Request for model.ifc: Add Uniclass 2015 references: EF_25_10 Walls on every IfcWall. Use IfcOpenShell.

First a look at what the model holds.

```python
import ifcopenshell

model = ifcopenshell.open("model.ifc")
print(model.schema)
print("classifications:", [c.Name for c in model.by_type("IfcClassification")])
for ifc_class in ("IfcDoor", "IfcRoof", "IfcStair", "IfcWall", "IfcWindow"):
    print(ifc_class, len(model.by_type(ifc_class)))
```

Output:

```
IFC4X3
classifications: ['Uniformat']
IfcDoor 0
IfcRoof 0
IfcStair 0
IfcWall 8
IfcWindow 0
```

```python
import ifcopenshell
import ifcopenshell.api.classification

model = ifcopenshell.open("model.ifc")

system = ifcopenshell.api.classification.add_classification(model, classification="Uniclass 2015")

codes = {
    "IfcWall": ("EF_25_10", "Walls"),
}
for ifc_class, (code, name) in codes.items():
    products = model.by_type(ifc_class)
    ifcopenshell.api.classification.add_reference(
        model, products=products, classification=system, identification=code, name=name
    )
    print(code, len(products))

model.write("model_v2.ifc")
```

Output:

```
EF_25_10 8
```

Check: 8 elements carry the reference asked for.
